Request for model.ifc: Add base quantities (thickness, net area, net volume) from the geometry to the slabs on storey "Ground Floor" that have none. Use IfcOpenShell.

First a look at what the model holds.

```python
import ifcopenshell
import ifcopenshell.util.element
import ifcopenshell.util.unit

model = ifcopenshell.open("model.ifc")
print(model.schema)
for unit_type in ("LENGTHUNIT", "AREAUNIT", "VOLUMEUNIT"):
    print(unit_type, ifcopenshell.util.unit.calculate_unit_scale(model, unit_type))
storey = next(s for s in model.by_type("IfcBuildingStorey") if s.Name == "Ground Floor")
slabs = [e for e in ifcopenshell.util.element.get_decomposition(storey) if e.is_a("IfcSlab")]
for e in sorted(slabs, key=lambda e: e.id()):
    print(e.id(), e.is_a(), e.Name, list(ifcopenshell.util.element.get_psets(e, qtos_only=True)), sep=" | ")
```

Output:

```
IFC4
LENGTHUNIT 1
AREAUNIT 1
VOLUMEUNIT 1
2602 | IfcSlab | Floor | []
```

```python
import ifcopenshell
import ifcopenshell.api.pset
import ifcopenshell.geom
import ifcopenshell.util.element
import ifcopenshell.util.shape
import ifcopenshell.util.unit

model = ifcopenshell.open("model.ifc")
unit_scale = ifcopenshell.util.unit.calculate_unit_scale(model)
area_scale = ifcopenshell.util.unit.calculate_unit_scale(model, "AREAUNIT")
volume_scale = ifcopenshell.util.unit.calculate_unit_scale(model, "VOLUMEUNIT")
settings = ifcopenshell.geom.settings()

storey = next(s for s in model.by_type("IfcBuildingStorey") if s.Name == "Ground Floor")
slabs = [e for e in ifcopenshell.util.element.get_decomposition(storey) if e.is_a("IfcSlab")]

for e in sorted(slabs, key=lambda e: e.id()):
    if ifcopenshell.util.element.get_psets(e, qtos_only=True, should_inherit=False):
        continue
    # Geometry comes back in metres, in the element's own axes.
    shape = ifcopenshell.geom.create_shape(settings, e)
    values = {
        "Width": ifcopenshell.util.shape.get_z(shape.geometry) / unit_scale,
        "NetArea": ifcopenshell.util.shape.get_footprint_area(shape.geometry) / area_scale,
        "NetVolume": ifcopenshell.util.shape.get_volume(shape.geometry) / volume_scale,
    }
    qto = ifcopenshell.api.pset.add_qto(model, product=e, name="Qto_SlabBaseQuantities")
    ifcopenshell.api.pset.edit_qto(model, qto=qto, properties=values)
    print(e.id(), {k: round(v, 3) for k, v in values.items()})

model.write("model_v2.ifc")
```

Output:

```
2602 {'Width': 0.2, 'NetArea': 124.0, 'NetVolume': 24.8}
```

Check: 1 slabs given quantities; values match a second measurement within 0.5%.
